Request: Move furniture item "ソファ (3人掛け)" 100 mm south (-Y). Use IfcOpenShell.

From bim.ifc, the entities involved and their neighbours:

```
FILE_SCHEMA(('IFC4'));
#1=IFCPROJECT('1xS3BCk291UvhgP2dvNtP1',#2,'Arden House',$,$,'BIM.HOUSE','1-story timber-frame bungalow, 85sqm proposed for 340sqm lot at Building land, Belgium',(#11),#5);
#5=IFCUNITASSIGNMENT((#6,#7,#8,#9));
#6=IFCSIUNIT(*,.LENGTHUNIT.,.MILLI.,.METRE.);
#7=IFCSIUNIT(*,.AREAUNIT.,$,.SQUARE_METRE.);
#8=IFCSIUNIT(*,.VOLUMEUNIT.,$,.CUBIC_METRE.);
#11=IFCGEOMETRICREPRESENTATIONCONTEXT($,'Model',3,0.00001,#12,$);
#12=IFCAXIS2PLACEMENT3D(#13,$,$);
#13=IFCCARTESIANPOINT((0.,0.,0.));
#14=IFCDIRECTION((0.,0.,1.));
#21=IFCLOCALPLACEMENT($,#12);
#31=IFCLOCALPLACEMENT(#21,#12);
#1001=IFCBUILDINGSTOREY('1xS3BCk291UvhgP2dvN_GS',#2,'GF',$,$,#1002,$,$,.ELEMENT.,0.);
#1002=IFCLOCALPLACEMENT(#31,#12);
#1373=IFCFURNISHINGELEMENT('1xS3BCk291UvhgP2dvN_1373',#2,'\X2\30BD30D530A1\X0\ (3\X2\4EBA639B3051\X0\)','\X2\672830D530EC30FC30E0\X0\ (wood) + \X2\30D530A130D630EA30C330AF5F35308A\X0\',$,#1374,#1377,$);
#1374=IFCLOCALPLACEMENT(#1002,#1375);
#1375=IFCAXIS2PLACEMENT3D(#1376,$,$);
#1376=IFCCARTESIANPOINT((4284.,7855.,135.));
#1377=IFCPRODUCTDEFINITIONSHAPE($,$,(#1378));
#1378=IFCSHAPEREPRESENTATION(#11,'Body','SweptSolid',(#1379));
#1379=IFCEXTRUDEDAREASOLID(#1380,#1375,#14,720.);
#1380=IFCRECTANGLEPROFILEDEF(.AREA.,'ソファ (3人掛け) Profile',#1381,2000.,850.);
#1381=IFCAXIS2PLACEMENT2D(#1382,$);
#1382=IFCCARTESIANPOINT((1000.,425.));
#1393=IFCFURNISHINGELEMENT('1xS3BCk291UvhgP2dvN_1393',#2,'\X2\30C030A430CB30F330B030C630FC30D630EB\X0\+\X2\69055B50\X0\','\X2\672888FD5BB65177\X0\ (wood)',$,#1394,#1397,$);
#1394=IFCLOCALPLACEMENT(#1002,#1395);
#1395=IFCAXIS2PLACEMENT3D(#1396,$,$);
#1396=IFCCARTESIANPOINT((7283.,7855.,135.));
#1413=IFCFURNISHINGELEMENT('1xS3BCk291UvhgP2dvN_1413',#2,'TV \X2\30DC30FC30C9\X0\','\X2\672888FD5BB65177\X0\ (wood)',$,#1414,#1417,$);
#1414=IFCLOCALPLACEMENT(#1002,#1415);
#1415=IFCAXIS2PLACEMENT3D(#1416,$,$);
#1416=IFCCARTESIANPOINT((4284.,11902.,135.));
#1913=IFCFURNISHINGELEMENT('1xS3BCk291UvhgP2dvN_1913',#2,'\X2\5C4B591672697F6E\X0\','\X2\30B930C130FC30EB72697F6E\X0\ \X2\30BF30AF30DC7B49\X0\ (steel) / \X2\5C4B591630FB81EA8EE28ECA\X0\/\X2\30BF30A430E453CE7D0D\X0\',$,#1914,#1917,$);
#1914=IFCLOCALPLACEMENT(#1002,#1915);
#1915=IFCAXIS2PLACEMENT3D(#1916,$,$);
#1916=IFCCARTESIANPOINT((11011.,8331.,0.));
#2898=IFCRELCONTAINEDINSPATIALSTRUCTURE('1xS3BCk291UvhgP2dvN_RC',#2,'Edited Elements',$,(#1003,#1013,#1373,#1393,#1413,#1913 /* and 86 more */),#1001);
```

```python
import ifcopenshell
import ifcopenshell.api.geometry
import ifcopenshell.util.placement
import ifcopenshell.util.unit

model = ifcopenshell.open("bim.ifc")
unit_scale = ifcopenshell.util.unit.calculate_unit_scale(model)

item = model.by_id(1373)
matrix = ifcopenshell.util.placement.get_local_placement(item.ObjectPlacement)
matrix[1, 3] -= 0.1 / unit_scale
ifcopenshell.api.geometry.edit_object_placement(model, product=item, matrix=matrix, is_si=False)

print(ifcopenshell.util.placement.get_local_placement(item.ObjectPlacement).round(3) + 0.0)

model.write("bim-out.ifc")
```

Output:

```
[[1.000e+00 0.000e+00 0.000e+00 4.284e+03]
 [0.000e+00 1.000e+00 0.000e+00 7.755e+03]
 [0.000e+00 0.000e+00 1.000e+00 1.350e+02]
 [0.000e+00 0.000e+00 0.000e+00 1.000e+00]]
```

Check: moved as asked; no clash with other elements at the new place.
